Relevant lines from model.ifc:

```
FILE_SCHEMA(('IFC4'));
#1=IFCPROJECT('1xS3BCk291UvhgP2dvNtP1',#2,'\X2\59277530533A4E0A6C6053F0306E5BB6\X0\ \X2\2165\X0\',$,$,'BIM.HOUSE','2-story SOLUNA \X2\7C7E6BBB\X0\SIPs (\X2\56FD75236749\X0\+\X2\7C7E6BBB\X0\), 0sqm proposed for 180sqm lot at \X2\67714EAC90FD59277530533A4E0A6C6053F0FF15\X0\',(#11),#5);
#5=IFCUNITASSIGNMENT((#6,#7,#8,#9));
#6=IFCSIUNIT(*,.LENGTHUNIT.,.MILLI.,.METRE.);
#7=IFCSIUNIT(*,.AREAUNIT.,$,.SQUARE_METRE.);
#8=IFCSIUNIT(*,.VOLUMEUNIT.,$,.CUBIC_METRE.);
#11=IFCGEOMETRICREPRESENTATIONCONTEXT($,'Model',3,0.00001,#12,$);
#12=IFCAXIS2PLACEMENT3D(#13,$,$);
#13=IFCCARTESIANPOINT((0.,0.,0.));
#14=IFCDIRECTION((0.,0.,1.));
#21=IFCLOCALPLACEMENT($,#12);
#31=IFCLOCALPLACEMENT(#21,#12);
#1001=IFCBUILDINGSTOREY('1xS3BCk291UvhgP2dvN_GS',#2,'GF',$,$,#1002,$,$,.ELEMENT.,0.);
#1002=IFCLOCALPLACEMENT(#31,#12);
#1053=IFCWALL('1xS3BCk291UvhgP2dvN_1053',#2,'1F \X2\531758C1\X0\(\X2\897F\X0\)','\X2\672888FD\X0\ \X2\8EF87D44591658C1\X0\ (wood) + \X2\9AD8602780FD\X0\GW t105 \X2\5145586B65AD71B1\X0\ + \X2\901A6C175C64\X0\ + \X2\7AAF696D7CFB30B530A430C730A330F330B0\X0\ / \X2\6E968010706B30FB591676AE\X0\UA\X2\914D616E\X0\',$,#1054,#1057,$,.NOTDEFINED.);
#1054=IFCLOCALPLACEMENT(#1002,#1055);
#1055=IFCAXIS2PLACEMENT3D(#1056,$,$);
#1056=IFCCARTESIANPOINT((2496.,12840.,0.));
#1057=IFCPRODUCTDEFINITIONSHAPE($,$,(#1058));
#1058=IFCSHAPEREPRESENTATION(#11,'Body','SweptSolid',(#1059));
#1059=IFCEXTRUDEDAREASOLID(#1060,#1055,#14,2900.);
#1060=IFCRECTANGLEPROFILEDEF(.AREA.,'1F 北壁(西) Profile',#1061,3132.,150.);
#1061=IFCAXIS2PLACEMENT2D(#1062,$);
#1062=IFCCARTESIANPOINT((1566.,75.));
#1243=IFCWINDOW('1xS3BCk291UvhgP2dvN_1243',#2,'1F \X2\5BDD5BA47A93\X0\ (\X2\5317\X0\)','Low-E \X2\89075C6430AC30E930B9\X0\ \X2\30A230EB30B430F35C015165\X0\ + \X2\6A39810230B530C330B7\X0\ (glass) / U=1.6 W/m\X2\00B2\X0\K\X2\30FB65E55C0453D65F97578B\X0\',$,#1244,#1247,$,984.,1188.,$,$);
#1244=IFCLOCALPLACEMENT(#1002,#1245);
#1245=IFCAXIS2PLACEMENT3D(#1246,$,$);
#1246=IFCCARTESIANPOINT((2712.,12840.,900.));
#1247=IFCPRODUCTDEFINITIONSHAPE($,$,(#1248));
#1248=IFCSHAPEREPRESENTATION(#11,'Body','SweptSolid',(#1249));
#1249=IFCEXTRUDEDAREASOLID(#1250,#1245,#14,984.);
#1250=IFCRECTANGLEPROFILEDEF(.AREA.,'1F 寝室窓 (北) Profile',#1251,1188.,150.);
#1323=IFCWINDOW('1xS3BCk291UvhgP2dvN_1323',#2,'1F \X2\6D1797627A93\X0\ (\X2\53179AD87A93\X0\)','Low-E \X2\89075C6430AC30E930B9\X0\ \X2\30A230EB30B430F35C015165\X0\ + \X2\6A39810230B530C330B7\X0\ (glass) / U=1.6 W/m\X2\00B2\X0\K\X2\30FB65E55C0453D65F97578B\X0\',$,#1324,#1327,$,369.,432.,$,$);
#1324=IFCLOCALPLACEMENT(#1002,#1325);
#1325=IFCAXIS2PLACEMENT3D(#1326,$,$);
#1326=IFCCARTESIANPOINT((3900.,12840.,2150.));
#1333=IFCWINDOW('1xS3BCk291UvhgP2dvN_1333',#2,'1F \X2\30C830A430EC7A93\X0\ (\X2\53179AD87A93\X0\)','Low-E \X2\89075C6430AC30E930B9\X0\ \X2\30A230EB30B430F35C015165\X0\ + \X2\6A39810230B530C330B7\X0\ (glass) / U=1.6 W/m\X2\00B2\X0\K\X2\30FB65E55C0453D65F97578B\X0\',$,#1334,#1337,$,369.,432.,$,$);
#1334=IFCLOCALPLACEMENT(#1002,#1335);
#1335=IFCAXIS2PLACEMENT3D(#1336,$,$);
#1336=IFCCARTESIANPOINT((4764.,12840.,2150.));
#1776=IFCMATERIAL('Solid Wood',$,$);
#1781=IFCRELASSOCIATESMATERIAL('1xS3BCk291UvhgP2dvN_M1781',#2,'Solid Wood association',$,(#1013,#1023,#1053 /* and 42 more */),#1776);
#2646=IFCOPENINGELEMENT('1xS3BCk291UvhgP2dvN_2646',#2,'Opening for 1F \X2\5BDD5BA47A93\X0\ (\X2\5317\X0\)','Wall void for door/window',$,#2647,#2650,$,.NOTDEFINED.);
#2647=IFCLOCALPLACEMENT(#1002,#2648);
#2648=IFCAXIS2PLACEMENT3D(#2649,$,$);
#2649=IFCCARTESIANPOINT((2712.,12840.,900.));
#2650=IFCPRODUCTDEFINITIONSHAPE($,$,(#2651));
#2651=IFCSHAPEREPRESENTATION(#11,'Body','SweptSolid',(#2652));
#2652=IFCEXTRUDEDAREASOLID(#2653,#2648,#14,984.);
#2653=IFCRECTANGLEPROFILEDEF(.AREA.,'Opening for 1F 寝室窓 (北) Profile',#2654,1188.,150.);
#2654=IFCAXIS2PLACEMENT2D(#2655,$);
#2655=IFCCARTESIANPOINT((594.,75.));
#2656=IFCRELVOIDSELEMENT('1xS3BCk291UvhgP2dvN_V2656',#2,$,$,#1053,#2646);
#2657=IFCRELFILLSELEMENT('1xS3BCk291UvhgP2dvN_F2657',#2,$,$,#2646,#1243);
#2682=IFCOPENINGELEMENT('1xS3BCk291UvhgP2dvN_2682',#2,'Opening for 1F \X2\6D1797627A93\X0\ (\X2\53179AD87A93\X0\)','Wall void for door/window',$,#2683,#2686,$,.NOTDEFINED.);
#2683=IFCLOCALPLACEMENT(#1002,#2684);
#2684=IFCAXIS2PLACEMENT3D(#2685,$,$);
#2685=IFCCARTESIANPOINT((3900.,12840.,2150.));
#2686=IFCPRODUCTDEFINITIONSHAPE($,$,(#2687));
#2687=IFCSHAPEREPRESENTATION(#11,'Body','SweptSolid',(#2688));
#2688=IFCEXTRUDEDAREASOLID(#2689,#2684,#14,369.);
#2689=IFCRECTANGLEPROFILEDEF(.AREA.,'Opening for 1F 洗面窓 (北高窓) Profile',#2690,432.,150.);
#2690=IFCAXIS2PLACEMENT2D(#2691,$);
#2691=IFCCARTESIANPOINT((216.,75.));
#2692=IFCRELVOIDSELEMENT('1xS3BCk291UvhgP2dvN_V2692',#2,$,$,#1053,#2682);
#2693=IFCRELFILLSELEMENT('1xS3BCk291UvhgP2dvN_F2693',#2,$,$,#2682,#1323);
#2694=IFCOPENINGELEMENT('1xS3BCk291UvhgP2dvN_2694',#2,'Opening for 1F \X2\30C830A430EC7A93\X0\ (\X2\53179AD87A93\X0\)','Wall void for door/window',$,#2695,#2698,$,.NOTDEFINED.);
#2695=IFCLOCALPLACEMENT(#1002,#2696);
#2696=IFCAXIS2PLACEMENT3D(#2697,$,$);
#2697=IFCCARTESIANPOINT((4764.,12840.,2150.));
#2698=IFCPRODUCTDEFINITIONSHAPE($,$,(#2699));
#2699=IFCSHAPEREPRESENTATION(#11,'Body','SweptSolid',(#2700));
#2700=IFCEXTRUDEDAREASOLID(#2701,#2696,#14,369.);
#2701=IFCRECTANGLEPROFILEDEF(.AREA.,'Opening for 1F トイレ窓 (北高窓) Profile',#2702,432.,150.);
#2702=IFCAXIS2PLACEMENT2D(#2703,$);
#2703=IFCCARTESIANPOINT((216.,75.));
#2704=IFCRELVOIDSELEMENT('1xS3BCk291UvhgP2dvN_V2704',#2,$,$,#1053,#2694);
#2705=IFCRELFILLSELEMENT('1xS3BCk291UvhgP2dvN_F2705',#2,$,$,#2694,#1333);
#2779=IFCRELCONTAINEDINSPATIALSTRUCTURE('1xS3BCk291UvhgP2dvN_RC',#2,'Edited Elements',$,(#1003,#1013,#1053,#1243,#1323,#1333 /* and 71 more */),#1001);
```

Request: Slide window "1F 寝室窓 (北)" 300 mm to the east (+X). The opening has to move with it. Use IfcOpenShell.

```python
import ifcopenshell
import ifcopenshell.api.geometry
import ifcopenshell.util.placement

model = ifcopenshell.open("model.ifc")

window = model.by_id(1243)
opening = window.FillsVoids[0].RelatingOpeningElement
wall = opening.VoidsElements[0].RelatingBuildingElement

wall_matrix = ifcopenshell.util.placement.get_local_placement(wall.ObjectPlacement)
shift = wall_matrix[:3, 0] * 300.0
before = ifcopenshell.util.placement.get_local_placement(window.ObjectPlacement)[:3, 3].copy()

# The window is not placed relative to its opening, so move both.
for product in (opening, window):
    matrix = ifcopenshell.util.placement.get_local_placement(product.ObjectPlacement)
    matrix[:3, 3] += shift
    ifcopenshell.api.geometry.edit_object_placement(model, product=product, matrix=matrix, is_si=False)

after = ifcopenshell.util.placement.get_local_placement(window.ObjectPlacement)[:3, 3]
print("window moved by", (after - before).round(3) + 0.0)

model.write("model_edited.ifc")
```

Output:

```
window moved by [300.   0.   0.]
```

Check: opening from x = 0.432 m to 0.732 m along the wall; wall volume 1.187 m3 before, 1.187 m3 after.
